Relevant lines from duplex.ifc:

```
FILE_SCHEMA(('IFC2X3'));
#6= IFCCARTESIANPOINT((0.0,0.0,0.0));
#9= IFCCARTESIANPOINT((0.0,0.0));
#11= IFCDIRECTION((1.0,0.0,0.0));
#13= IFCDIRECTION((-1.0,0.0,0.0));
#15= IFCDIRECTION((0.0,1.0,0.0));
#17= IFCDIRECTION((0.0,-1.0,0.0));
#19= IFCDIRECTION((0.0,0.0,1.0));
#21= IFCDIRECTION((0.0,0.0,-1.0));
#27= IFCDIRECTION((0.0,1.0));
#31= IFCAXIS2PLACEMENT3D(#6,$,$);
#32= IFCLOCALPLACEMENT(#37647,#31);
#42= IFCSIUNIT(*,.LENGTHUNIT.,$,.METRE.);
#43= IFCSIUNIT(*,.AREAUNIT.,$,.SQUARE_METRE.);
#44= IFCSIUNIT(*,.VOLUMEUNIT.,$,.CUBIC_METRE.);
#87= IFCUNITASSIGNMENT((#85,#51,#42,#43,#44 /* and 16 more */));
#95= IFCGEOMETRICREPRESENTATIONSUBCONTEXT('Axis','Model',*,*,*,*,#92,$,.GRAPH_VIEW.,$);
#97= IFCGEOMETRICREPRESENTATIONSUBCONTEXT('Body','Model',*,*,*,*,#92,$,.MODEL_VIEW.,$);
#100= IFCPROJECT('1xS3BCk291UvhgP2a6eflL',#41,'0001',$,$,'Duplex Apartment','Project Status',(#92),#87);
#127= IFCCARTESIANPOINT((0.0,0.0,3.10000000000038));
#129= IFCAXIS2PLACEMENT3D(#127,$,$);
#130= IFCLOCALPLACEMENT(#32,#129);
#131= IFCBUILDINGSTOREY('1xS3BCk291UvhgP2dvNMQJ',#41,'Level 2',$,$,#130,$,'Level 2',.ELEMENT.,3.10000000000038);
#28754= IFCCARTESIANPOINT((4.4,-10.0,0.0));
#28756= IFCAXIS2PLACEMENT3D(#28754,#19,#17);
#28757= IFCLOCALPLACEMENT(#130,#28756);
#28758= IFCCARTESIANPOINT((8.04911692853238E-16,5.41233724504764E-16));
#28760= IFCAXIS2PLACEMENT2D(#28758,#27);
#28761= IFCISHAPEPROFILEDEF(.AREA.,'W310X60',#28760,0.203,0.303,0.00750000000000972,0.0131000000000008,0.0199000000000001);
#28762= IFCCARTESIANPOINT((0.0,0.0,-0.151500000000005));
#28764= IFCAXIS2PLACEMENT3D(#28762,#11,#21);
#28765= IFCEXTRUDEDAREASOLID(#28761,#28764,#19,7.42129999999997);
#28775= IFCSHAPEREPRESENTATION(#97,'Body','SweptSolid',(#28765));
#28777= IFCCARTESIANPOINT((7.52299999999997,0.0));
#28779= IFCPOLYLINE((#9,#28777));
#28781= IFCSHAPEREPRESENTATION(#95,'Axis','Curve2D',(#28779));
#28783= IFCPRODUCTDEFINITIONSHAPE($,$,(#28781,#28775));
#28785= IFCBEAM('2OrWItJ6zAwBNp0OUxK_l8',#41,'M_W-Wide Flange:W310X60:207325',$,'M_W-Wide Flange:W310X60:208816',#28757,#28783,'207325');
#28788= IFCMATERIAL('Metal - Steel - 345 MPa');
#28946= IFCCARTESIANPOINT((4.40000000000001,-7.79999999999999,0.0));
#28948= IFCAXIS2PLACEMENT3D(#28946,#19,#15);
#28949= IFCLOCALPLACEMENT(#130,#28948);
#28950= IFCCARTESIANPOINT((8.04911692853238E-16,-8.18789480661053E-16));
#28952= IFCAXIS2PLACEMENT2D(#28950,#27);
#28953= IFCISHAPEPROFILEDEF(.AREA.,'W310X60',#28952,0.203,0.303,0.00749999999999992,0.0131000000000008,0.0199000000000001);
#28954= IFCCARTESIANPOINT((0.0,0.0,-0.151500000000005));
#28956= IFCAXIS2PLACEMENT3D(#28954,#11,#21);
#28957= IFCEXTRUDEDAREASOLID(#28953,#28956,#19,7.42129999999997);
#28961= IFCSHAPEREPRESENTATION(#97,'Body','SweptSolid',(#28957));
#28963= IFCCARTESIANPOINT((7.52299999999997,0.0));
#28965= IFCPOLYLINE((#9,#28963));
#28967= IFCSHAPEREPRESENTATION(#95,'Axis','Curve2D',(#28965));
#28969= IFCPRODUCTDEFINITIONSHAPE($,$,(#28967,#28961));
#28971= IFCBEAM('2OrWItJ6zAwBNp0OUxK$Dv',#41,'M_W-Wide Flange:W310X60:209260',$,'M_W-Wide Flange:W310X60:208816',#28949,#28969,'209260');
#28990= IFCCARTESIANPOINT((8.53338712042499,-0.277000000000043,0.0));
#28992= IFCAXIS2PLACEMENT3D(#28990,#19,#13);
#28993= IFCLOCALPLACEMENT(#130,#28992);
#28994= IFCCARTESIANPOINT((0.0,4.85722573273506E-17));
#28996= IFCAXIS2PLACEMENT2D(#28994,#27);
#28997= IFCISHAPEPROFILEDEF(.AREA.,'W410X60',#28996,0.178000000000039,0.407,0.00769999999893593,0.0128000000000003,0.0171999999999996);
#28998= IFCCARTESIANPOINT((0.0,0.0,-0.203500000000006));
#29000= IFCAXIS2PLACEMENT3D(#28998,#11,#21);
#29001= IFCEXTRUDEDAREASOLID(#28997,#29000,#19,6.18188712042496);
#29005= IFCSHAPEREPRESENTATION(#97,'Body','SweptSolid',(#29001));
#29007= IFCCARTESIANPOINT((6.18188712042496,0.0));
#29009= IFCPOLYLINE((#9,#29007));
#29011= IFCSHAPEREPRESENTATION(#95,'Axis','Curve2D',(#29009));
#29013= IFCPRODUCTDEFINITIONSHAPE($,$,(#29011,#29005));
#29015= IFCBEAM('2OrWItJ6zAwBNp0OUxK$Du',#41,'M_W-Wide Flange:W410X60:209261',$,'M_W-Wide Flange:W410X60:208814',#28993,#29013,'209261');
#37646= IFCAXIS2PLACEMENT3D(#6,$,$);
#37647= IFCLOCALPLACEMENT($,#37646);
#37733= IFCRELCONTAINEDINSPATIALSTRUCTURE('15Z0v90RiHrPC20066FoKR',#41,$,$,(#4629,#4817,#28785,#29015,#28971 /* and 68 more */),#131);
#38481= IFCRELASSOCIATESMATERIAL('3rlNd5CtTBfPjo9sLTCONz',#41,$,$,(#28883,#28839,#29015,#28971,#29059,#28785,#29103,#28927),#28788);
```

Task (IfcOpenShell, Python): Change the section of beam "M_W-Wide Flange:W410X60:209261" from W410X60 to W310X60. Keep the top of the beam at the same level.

```python
import ifcopenshell
import ifcopenshell.util.element
import ifcopenshell.util.representation

model = ifcopenshell.open("duplex.ifc")

member = model.by_guid("2OrWItJ6zAwBNp0OUxK$Du")
source = next(p for p in model.by_type("IfcIShapeProfileDef") if p.ProfileName == "W310X60")

body = ifcopenshell.util.representation.get_representation(member, "Model", "Body")
solid = body.Items[0]
old_profile = solid.SweptArea

# Copy the section's sizes but keep this member's own profile position.
profile = ifcopenshell.util.element.copy(model, source)
# Profiles are centred, so shift by half the change in depth to hold the top.
shift = (old_profile.OverallDepth - profile.OverallDepth) / 2
x, y = old_profile.Position.Location.Coordinates
up = (-1.0, 0.0)  # upwards, in the solid's own plane
location = model.createIfcCartesianPoint((x + up[0] * shift, y + up[1] * shift))
profile.Position = model.createIfcAxis2Placement2D(location, old_profile.Position.RefDirection)
solid.SweptArea = profile
if not model.get_total_inverses(old_profile):
    ifcopenshell.util.element.remove_deep2(model, old_profile)
member.Name = member.Name.replace("W410X60", "W310X60")
member.ObjectType = member.ObjectType.replace("W410X60", "W310X60")

print(solid.SweptArea)

model.write("duplex_v2.ifc")
```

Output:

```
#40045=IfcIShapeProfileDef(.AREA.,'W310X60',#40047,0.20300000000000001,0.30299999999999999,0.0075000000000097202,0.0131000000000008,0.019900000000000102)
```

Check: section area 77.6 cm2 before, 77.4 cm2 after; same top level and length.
